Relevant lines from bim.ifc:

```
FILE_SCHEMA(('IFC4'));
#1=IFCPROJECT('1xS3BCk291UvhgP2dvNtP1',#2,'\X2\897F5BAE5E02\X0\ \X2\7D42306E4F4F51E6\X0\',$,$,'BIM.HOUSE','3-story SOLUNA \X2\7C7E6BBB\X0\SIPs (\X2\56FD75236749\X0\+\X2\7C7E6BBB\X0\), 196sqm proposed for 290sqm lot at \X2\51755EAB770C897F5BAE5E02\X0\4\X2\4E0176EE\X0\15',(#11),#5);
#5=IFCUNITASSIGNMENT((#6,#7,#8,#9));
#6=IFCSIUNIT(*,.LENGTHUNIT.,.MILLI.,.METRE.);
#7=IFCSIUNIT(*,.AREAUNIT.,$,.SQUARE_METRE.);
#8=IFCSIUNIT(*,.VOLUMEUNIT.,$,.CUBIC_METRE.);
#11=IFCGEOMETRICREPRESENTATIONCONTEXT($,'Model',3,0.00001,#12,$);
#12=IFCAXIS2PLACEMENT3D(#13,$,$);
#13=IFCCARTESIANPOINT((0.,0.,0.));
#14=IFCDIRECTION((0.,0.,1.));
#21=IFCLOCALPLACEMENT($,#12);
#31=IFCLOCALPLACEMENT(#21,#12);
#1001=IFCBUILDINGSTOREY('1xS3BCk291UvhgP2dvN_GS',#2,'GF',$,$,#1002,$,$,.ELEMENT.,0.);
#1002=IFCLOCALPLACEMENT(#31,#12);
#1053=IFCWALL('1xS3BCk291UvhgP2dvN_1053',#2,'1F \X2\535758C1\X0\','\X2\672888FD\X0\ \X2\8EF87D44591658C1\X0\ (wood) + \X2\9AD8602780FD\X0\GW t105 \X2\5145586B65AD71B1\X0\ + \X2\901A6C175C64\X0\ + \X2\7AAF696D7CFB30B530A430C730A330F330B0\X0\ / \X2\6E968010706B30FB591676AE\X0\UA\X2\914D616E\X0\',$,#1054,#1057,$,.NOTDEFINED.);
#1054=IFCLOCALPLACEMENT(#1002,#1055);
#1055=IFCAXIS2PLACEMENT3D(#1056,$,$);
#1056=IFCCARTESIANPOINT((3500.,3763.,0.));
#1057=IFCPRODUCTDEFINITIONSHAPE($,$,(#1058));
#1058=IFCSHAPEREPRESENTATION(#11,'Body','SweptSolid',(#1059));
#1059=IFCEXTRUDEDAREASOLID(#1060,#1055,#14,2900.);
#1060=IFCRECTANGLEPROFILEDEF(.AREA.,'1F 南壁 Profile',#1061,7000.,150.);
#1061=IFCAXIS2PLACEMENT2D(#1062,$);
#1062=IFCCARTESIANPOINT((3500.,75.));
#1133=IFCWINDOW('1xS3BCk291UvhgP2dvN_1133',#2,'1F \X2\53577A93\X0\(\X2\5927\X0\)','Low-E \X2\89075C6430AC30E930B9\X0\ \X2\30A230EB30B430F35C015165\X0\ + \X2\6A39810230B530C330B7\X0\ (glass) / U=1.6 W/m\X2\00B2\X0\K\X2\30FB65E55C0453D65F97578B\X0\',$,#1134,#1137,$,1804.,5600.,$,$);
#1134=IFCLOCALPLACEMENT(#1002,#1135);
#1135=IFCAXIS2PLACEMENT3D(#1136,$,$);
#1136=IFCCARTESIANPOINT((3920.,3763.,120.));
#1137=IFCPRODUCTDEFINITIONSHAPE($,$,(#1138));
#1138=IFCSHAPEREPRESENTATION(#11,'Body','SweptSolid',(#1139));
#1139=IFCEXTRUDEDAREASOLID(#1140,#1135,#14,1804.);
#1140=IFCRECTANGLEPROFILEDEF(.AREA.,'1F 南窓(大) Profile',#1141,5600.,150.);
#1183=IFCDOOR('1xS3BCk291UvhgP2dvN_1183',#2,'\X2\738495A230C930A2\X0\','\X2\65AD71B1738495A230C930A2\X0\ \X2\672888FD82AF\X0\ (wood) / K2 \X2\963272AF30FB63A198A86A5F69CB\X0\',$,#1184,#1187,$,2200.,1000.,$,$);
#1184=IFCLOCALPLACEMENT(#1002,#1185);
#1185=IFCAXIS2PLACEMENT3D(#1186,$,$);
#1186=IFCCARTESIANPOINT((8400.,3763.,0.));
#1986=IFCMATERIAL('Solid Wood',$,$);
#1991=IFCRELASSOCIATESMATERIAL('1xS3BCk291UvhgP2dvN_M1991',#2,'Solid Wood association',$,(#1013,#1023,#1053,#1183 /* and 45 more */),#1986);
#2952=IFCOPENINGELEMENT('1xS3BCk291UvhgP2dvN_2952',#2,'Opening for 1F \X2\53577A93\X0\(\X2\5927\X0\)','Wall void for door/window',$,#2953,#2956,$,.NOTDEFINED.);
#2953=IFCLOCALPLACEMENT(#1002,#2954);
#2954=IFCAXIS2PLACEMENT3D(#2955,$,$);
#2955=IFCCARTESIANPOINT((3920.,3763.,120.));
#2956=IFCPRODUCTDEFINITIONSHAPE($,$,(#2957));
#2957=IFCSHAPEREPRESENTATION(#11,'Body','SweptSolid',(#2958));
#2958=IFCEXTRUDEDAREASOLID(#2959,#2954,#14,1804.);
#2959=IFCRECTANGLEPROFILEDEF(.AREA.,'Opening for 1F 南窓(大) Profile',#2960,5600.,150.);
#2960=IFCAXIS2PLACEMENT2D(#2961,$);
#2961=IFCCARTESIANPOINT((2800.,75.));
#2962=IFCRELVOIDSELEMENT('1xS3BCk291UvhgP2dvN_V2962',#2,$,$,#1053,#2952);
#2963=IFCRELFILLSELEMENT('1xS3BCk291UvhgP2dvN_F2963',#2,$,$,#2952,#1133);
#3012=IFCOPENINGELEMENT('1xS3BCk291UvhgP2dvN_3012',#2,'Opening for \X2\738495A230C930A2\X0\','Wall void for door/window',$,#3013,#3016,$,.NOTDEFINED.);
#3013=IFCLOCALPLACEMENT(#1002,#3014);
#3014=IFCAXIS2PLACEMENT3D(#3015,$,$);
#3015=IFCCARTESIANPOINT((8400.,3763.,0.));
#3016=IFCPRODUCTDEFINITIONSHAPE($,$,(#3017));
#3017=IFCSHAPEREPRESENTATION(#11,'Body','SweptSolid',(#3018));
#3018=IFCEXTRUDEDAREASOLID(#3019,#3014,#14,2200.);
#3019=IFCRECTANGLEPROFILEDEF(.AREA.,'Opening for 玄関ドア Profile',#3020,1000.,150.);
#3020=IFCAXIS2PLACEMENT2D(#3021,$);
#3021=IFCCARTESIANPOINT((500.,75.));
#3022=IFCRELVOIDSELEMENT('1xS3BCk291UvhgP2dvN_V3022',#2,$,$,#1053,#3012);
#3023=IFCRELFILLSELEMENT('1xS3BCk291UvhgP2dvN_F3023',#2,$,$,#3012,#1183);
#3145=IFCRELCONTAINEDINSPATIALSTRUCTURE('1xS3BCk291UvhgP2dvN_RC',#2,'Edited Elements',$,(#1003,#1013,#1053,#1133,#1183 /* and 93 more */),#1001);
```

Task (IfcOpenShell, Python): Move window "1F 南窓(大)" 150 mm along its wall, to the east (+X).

```python
import ifcopenshell
import ifcopenshell.api.geometry
import ifcopenshell.util.placement
import ifcopenshell.util.unit

model = ifcopenshell.open("bim.ifc")
unit_scale = ifcopenshell.util.unit.calculate_unit_scale(model)

window = model.by_id(1133)
opening = window.FillsVoids[0].RelatingOpeningElement
wall = opening.VoidsElements[0].RelatingBuildingElement

wall_matrix = ifcopenshell.util.placement.get_local_placement(wall.ObjectPlacement)
shift = wall_matrix[:3, 0] * 0.15 / unit_scale
before = ifcopenshell.util.placement.get_local_placement(window.ObjectPlacement)[:3, 3].copy()

# The window is not placed relative to its opening, so move both.
for product in (opening, window):
    matrix = ifcopenshell.util.placement.get_local_placement(product.ObjectPlacement)
    matrix[:3, 3] += shift
    ifcopenshell.api.geometry.edit_object_placement(model, product=product, matrix=matrix, is_si=False)

after = ifcopenshell.util.placement.get_local_placement(window.ObjectPlacement)[:3, 3]
print("window moved by", (after - before).round(3) + 0.0)

model.write("bim-out.ifc")
```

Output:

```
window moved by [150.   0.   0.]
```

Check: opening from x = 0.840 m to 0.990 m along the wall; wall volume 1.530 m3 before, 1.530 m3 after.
